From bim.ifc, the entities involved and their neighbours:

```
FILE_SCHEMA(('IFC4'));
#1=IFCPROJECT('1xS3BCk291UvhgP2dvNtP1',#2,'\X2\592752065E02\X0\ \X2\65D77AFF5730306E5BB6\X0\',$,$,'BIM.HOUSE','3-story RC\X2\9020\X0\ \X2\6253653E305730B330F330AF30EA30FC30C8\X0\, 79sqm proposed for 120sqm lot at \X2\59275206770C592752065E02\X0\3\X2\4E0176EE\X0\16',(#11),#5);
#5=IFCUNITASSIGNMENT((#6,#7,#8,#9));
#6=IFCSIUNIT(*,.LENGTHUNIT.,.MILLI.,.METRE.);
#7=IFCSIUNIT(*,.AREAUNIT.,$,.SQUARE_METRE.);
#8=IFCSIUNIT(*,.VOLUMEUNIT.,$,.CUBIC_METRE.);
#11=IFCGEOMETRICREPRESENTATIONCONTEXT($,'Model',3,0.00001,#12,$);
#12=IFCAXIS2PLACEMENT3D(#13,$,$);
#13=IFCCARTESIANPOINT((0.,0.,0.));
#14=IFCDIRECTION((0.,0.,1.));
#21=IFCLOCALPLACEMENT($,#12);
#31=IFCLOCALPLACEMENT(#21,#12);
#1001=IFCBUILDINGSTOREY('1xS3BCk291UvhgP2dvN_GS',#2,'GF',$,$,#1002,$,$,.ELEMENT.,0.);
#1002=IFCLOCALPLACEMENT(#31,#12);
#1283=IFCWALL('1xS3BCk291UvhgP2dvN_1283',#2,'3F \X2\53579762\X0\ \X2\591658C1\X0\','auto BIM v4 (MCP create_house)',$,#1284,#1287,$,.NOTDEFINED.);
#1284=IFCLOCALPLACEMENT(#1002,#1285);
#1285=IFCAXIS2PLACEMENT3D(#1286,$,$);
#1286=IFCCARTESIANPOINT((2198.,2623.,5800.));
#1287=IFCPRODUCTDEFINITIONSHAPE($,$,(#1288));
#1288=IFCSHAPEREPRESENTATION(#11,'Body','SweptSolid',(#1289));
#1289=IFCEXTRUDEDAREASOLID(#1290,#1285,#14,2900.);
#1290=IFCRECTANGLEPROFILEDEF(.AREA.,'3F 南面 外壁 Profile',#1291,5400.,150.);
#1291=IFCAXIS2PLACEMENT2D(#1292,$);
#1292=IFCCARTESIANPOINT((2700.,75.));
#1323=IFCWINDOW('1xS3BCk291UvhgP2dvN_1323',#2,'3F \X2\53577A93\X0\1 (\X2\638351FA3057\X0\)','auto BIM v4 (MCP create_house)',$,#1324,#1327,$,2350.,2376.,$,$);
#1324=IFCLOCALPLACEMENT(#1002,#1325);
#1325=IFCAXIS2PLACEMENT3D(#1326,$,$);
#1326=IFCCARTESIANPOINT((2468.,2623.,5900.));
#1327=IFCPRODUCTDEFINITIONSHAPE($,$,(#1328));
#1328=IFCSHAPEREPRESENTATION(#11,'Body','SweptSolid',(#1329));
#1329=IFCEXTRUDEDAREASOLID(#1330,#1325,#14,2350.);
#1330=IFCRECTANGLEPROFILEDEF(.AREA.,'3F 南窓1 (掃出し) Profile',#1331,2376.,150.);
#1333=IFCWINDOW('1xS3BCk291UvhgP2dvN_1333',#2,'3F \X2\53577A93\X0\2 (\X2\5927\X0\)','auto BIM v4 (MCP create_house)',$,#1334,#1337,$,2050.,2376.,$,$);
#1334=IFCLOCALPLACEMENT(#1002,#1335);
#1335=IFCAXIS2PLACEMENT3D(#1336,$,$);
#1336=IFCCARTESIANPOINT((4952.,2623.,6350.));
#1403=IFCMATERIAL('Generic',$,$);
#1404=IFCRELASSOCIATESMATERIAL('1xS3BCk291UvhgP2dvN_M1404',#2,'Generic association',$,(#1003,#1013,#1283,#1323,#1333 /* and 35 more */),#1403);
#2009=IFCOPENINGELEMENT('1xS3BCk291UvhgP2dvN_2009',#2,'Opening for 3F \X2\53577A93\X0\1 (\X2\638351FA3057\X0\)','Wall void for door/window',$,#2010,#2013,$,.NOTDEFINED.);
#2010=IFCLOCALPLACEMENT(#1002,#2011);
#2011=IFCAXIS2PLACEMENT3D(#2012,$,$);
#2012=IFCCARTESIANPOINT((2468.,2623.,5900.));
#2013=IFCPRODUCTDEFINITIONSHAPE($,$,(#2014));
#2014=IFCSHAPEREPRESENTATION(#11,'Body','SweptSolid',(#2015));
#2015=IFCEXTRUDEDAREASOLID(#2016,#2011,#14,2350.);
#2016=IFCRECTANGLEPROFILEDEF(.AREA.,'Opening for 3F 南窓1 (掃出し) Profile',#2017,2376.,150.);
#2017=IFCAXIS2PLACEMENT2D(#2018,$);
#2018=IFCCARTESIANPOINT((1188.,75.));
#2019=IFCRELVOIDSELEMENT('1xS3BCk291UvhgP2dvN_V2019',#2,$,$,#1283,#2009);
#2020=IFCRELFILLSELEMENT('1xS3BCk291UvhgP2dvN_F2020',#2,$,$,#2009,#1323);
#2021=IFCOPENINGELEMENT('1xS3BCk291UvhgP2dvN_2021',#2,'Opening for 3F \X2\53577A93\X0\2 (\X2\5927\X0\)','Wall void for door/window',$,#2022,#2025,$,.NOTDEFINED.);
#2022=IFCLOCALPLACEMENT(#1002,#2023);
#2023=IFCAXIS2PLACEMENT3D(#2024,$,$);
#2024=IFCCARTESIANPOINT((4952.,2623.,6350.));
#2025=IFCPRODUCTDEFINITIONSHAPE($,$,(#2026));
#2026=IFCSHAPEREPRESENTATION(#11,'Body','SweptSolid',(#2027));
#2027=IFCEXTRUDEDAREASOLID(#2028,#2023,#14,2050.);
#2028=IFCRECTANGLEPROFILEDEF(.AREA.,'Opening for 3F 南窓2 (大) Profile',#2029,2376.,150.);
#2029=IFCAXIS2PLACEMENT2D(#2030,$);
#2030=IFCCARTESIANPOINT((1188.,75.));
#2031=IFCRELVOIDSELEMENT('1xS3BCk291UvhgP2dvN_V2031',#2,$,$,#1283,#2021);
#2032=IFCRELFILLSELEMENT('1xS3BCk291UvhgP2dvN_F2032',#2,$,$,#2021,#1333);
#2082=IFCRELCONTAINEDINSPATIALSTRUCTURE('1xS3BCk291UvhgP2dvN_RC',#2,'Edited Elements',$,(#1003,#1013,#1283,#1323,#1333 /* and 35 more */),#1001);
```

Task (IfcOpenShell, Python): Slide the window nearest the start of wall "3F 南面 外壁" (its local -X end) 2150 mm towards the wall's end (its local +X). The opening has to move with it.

```python
import ifcopenshell
import ifcopenshell.api.geometry
import ifcopenshell.util.placement
import ifcopenshell.util.unit

model = ifcopenshell.open("bim.ifc")
unit_scale = ifcopenshell.util.unit.calculate_unit_scale(model)

window = model.by_id(1323)
opening = window.FillsVoids[0].RelatingOpeningElement
wall = opening.VoidsElements[0].RelatingBuildingElement

wall_matrix = ifcopenshell.util.placement.get_local_placement(wall.ObjectPlacement)
shift = wall_matrix[:3, 0] * 2.15 / unit_scale
before = ifcopenshell.util.placement.get_local_placement(window.ObjectPlacement)[:3, 3].copy()

# The window is not placed relative to its opening, so move both.
for product in (opening, window):
    matrix = ifcopenshell.util.placement.get_local_placement(product.ObjectPlacement)
    matrix[:3, 3] += shift
    ifcopenshell.api.geometry.edit_object_placement(model, product=product, matrix=matrix, is_si=False)

after = ifcopenshell.util.placement.get_local_placement(window.ObjectPlacement)[:3, 3]
print("window moved by", (after - before).round(3) + 0.0)

model.write("bim_v2.ifc")
```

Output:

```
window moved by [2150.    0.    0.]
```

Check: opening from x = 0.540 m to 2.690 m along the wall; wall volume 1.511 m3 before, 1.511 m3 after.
